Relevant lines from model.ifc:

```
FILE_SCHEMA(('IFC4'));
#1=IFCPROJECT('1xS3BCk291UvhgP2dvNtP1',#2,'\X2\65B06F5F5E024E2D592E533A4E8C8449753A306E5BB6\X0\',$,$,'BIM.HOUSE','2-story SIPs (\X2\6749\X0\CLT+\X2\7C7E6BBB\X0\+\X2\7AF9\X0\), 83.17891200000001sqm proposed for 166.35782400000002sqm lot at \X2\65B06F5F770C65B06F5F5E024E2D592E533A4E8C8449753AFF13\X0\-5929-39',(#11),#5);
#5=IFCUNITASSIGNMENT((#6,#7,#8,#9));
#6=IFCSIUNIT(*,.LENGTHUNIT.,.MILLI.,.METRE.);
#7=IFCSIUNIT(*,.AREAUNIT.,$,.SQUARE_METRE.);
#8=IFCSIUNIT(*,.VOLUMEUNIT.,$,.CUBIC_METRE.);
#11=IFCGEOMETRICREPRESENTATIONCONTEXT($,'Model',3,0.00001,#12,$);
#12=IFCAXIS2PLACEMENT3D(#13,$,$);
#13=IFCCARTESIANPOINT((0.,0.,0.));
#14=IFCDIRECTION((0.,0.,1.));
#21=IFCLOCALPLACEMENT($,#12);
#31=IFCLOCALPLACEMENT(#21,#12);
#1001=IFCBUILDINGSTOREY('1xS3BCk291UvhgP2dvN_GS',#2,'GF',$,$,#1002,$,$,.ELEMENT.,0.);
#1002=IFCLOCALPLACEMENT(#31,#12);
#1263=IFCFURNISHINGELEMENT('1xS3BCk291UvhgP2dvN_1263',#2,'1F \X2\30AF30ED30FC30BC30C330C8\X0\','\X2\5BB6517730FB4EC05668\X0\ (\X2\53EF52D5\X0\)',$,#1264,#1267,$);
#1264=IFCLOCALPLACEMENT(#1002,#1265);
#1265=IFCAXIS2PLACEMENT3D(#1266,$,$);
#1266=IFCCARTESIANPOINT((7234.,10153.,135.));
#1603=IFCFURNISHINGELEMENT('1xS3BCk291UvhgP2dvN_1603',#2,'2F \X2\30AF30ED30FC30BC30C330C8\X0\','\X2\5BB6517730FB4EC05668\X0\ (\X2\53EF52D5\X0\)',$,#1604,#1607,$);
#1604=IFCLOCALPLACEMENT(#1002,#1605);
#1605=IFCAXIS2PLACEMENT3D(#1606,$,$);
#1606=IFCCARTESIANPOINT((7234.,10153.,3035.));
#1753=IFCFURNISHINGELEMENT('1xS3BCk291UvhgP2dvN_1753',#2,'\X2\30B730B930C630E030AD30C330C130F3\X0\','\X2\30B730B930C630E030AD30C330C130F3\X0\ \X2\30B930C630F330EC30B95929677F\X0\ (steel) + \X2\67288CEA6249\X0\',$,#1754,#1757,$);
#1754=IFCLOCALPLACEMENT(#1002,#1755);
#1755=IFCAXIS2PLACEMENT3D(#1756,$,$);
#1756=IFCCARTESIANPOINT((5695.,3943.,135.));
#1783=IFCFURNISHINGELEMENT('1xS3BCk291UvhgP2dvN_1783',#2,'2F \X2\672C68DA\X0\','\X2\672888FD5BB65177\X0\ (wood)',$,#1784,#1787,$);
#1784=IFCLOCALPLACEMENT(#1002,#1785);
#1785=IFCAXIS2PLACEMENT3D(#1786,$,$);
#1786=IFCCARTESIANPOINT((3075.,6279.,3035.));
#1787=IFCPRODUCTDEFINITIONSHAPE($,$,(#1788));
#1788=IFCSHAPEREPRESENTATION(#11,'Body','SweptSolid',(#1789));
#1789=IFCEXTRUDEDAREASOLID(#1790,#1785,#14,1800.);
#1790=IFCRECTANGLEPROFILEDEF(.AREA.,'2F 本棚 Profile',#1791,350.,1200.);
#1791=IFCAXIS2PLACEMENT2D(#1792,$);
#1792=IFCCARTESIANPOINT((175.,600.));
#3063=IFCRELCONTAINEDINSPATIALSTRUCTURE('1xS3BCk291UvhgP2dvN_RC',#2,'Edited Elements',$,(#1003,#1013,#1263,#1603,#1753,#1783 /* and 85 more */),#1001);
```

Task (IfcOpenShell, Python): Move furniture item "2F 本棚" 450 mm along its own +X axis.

```python
import ifcopenshell
import ifcopenshell.api.geometry
import ifcopenshell.util.placement
import ifcopenshell.util.unit

model = ifcopenshell.open("model.ifc")
unit_scale = ifcopenshell.util.unit.calculate_unit_scale(model)

item = model.by_guid("1xS3BCk291UvhgP2dvN_1783")
matrix = ifcopenshell.util.placement.get_local_placement(item.ObjectPlacement)
matrix[:3, 3] += matrix[:3, 0] * 0.45 / unit_scale
ifcopenshell.api.geometry.edit_object_placement(model, product=item, matrix=matrix, is_si=False)

print(ifcopenshell.util.placement.get_local_placement(item.ObjectPlacement).round(3) + 0.0)

model.write("model_edited.ifc")
```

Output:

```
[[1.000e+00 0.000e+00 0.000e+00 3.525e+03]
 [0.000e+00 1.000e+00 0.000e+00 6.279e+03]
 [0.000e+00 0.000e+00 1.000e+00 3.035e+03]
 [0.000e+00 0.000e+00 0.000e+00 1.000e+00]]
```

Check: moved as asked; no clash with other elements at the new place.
